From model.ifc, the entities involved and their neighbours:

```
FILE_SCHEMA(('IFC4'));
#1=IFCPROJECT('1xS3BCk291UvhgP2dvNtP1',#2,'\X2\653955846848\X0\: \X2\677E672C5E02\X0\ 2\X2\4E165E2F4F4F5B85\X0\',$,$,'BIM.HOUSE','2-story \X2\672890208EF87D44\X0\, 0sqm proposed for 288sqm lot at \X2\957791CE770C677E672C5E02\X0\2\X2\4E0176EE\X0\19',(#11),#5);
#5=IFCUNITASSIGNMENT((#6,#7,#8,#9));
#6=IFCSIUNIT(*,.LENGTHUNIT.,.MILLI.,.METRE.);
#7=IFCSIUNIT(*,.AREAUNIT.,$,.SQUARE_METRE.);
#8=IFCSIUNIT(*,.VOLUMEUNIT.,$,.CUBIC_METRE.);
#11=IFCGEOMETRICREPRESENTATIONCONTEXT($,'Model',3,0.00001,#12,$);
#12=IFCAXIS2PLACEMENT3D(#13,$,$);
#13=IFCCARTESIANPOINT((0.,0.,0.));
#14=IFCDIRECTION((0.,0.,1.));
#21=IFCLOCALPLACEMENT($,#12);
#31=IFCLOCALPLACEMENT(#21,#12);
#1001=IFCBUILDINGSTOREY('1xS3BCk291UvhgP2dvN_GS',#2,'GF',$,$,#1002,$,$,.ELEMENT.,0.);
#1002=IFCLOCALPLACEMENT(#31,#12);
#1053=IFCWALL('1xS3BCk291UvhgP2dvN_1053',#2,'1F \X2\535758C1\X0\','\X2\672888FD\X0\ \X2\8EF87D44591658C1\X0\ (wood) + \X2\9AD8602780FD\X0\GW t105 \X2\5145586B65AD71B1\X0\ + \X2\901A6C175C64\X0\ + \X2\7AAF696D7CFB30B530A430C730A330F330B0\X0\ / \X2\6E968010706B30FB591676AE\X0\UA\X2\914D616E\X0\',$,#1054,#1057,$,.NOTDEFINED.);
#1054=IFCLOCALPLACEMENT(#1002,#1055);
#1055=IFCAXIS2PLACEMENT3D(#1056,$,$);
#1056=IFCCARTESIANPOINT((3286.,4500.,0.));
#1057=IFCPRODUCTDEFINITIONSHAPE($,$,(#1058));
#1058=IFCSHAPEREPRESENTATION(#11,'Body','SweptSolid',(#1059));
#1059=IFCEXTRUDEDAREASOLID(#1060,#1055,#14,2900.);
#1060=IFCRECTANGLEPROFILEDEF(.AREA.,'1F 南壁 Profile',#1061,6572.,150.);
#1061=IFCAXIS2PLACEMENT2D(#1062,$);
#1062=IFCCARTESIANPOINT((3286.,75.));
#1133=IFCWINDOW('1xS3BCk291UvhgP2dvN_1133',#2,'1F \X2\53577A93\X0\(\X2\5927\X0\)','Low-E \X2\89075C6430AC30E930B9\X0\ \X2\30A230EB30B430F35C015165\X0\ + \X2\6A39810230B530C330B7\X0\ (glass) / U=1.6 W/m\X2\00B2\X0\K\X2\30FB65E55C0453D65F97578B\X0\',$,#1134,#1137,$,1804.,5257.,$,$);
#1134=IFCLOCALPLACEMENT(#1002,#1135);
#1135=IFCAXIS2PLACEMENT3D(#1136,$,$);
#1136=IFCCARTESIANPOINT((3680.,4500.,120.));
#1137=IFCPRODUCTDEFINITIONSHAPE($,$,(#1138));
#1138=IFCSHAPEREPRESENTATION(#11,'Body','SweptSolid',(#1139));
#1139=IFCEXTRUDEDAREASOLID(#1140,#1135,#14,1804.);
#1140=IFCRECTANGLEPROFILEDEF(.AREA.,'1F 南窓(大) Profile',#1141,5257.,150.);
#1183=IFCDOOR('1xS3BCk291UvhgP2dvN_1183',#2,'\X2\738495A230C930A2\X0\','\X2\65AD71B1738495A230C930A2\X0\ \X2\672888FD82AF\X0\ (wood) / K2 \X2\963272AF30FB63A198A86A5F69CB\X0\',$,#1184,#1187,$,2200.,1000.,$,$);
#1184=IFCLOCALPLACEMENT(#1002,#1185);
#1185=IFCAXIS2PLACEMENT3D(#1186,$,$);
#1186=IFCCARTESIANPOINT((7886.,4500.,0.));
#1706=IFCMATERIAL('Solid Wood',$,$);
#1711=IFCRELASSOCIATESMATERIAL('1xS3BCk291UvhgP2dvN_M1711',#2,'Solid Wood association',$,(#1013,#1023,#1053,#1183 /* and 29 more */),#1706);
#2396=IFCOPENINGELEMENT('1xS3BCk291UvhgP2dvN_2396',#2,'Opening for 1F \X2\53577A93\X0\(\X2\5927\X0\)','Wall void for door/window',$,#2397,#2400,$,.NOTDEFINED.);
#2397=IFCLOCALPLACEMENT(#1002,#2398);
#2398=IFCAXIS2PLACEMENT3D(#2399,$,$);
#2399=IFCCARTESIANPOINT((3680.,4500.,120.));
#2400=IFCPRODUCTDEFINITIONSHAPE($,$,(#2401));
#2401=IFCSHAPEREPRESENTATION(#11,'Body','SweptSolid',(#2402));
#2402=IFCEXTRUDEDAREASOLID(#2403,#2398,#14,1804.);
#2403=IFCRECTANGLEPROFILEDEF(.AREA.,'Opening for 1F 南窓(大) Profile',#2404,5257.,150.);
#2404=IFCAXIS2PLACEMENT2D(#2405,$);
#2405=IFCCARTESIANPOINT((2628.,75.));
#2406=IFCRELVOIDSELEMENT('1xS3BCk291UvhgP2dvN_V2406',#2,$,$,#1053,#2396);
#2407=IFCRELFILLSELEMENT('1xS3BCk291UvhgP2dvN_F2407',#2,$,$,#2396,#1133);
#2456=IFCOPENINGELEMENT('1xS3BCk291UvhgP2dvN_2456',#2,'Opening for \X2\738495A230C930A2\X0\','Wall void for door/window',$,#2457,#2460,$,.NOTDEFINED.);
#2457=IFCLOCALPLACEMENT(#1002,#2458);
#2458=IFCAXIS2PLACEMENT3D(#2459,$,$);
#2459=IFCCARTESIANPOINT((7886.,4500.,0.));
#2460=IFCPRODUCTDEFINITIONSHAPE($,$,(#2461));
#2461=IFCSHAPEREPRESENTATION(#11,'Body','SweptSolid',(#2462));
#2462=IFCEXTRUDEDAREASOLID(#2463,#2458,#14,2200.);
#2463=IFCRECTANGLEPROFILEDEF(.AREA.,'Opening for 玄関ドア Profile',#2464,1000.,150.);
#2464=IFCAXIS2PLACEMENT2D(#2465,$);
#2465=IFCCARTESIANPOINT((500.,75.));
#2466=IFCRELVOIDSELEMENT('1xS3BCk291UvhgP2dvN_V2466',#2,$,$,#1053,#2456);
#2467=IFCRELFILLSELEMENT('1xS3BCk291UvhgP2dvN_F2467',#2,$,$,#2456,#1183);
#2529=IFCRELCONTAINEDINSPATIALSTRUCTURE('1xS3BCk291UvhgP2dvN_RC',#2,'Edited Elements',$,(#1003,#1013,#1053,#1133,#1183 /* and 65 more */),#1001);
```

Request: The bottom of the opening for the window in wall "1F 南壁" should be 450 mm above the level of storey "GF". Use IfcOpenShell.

```python
import numpy as np
import ifcopenshell
import ifcopenshell.api.geometry
import ifcopenshell.geom
import ifcopenshell.util.element
import ifcopenshell.util.placement
import ifcopenshell.util.shape
import ifcopenshell.util.unit

model = ifcopenshell.open("model.ifc")
unit_scale = ifcopenshell.util.unit.calculate_unit_scale(model)

window = model.by_guid("1xS3BCk291UvhgP2dvN_1133")
opening = window.FillsVoids[0].RelatingOpeningElement
storey = ifcopenshell.util.element.get_container(window, ifc_class="IfcBuildingStorey")
level = ifcopenshell.util.placement.get_local_placement(storey.ObjectPlacement)[2, 3]

# The opening's origin need not be at the sill, so measure its lowest point.
shape = ifcopenshell.geom.create_shape(ifcopenshell.geom.settings(), opening)
bottom = ifcopenshell.util.shape.get_shape_bottom_elevation(shape, shape.geometry) / unit_scale
dz = level + 0.45 / unit_scale - bottom

shift = np.array([0.0, 0.0, dz])
# The window is not placed relative to its opening, so move both.
for product in (opening, window):
    matrix = ifcopenshell.util.placement.get_local_placement(product.ObjectPlacement)
    matrix[:3, 3] += shift
    ifcopenshell.api.geometry.edit_object_placement(model, product=product, matrix=matrix, is_si=False)

print(f"moved by {dz * unit_scale:+.3f} m")

model.write("model-out.ifc")
```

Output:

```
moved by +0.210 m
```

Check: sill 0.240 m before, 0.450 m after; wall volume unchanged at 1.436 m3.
